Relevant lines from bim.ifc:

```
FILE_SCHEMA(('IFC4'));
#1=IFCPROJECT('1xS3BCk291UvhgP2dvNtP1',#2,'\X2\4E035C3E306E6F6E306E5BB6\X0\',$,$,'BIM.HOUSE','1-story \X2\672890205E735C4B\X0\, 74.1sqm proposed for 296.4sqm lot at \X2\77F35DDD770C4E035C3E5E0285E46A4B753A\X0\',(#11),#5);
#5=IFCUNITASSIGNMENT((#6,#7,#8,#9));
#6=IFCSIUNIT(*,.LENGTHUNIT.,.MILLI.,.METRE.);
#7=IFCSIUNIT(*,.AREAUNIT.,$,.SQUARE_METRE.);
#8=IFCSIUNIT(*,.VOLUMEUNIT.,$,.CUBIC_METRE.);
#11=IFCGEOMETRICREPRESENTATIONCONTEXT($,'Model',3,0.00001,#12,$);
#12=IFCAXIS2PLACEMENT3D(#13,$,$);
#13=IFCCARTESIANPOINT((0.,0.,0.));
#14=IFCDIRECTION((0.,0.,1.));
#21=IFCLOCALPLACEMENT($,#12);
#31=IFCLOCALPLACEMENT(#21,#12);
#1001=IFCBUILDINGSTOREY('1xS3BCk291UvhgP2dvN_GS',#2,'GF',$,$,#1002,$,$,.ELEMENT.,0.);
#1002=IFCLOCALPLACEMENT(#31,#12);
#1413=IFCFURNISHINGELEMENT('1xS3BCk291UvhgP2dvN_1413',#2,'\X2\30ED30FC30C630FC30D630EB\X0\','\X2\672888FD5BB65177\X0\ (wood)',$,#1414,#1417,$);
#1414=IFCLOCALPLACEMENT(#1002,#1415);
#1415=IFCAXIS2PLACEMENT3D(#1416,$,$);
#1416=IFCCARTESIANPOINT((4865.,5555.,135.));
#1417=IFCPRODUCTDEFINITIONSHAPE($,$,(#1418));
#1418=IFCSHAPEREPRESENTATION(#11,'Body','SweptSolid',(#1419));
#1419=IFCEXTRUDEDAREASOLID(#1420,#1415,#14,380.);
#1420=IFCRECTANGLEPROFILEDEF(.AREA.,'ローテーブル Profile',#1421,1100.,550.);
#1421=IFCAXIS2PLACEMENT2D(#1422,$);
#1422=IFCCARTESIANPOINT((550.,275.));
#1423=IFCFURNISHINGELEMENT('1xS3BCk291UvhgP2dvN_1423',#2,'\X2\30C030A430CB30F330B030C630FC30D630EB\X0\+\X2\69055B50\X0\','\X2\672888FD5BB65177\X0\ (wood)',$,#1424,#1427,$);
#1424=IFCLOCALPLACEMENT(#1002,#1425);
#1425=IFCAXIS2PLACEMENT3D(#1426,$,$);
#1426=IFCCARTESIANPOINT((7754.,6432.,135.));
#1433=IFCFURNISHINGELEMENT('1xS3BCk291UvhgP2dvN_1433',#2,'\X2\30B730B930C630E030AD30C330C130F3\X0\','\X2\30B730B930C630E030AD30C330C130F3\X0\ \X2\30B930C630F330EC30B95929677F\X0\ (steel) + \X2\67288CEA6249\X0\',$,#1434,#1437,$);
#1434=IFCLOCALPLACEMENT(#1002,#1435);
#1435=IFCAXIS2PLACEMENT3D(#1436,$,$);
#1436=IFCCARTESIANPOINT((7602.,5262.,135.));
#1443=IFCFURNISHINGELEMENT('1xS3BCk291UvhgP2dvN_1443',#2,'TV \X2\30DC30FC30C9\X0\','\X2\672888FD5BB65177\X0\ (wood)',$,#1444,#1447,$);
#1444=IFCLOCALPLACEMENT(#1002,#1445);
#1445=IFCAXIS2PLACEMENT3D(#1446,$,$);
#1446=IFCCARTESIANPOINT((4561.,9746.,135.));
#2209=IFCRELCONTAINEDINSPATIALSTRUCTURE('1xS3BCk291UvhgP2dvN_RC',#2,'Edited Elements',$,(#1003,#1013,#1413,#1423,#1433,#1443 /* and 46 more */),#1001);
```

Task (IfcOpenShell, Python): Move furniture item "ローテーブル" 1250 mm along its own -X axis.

```python
import ifcopenshell
import ifcopenshell.api.geometry
import ifcopenshell.util.placement
import ifcopenshell.util.unit

model = ifcopenshell.open("bim.ifc")
unit_scale = ifcopenshell.util.unit.calculate_unit_scale(model)

item = model.by_id(1413)
matrix = ifcopenshell.util.placement.get_local_placement(item.ObjectPlacement)
matrix[:3, 3] -= matrix[:3, 0] * 1.25 / unit_scale
ifcopenshell.api.geometry.edit_object_placement(model, product=item, matrix=matrix, is_si=False)

print(ifcopenshell.util.placement.get_local_placement(item.ObjectPlacement).round(3) + 0.0)

model.write("bim_edited.ifc")
```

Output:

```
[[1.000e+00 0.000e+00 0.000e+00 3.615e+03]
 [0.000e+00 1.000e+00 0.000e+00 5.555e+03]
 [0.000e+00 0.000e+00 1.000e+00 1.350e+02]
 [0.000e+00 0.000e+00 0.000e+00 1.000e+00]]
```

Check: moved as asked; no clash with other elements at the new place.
